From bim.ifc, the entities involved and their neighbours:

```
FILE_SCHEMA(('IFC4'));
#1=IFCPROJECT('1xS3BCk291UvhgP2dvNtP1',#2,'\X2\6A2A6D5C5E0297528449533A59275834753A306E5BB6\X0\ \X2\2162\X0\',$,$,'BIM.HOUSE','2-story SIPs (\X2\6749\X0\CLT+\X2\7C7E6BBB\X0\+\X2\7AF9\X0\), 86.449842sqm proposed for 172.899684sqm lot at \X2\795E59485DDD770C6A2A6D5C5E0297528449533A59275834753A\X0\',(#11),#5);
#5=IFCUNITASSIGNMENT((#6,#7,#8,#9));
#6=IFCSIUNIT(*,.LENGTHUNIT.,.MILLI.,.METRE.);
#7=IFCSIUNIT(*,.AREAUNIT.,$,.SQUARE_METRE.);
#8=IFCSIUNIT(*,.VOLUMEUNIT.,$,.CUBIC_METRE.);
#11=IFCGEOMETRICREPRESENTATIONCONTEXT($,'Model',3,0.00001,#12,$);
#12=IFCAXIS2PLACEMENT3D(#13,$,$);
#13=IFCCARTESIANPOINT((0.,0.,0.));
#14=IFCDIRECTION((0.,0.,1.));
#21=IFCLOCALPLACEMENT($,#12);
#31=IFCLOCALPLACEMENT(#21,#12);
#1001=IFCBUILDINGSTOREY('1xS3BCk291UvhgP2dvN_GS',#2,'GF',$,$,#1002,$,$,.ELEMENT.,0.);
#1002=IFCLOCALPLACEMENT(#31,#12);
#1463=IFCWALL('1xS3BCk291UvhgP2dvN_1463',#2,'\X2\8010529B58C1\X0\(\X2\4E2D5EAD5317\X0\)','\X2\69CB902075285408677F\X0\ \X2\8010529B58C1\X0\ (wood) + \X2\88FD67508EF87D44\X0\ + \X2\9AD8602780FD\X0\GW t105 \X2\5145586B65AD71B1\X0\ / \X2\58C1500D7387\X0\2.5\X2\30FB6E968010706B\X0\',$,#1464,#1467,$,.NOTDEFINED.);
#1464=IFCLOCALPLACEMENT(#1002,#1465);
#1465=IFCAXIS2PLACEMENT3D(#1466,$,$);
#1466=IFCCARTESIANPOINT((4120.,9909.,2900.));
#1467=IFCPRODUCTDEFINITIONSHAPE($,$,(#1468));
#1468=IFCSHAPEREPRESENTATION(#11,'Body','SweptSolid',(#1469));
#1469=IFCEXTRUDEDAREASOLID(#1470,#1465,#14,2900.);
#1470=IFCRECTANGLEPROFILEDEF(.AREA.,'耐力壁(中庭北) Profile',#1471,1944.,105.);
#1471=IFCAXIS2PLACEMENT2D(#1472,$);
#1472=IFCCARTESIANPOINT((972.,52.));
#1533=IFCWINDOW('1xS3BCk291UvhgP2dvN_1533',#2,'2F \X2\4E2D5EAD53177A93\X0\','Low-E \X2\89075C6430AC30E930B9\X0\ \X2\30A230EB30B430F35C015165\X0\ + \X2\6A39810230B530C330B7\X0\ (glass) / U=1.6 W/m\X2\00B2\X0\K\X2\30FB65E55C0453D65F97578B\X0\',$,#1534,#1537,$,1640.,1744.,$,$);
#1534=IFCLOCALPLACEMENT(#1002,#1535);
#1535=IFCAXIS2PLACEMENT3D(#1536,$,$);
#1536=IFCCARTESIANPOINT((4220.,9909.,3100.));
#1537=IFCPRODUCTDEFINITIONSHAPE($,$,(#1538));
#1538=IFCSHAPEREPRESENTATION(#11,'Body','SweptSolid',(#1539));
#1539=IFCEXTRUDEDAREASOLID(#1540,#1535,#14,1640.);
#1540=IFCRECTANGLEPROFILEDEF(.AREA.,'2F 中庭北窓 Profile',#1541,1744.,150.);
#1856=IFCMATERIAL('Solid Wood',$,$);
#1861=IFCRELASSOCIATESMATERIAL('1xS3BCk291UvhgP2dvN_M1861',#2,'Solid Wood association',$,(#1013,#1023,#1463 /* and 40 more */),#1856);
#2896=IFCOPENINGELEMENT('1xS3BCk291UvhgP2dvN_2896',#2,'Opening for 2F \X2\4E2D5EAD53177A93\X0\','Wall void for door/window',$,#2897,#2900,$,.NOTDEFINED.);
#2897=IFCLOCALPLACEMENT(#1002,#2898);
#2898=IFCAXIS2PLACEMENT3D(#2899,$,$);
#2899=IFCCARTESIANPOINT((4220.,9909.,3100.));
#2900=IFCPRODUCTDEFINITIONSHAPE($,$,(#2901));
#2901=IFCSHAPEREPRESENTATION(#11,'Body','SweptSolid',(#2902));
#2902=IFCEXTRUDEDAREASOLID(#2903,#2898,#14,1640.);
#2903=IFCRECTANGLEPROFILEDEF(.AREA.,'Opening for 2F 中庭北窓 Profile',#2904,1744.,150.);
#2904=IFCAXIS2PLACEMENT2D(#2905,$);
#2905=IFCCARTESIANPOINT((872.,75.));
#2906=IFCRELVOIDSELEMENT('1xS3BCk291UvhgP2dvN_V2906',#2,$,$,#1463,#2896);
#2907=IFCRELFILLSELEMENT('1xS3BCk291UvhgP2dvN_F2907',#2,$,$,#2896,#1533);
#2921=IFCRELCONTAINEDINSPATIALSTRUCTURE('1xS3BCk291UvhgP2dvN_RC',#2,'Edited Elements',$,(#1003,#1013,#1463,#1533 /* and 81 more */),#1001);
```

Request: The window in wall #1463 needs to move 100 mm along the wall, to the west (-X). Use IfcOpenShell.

```python
import ifcopenshell
import ifcopenshell.api.geometry
import ifcopenshell.util.placement

model = ifcopenshell.open("bim.ifc")

window = model.by_id(1533)
opening = window.FillsVoids[0].RelatingOpeningElement
wall = opening.VoidsElements[0].RelatingBuildingElement

wall_matrix = ifcopenshell.util.placement.get_local_placement(wall.ObjectPlacement)
shift = wall_matrix[:3, 0] * -100.0
before = ifcopenshell.util.placement.get_local_placement(window.ObjectPlacement)[:3, 3].copy()

# The window is not placed relative to its opening, so move both.
for product in (opening, window):
    matrix = ifcopenshell.util.placement.get_local_placement(product.ObjectPlacement)
    matrix[:3, 3] += shift
    ifcopenshell.api.geometry.edit_object_placement(model, product=product, matrix=matrix, is_si=False)

after = ifcopenshell.util.placement.get_local_placement(window.ObjectPlacement)[:3, 3]
print("window moved by", (after - before).round(3) + 0.0)

model.write("bim_edited.ifc")
```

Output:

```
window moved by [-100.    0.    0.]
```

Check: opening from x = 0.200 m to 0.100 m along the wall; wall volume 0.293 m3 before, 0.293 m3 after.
